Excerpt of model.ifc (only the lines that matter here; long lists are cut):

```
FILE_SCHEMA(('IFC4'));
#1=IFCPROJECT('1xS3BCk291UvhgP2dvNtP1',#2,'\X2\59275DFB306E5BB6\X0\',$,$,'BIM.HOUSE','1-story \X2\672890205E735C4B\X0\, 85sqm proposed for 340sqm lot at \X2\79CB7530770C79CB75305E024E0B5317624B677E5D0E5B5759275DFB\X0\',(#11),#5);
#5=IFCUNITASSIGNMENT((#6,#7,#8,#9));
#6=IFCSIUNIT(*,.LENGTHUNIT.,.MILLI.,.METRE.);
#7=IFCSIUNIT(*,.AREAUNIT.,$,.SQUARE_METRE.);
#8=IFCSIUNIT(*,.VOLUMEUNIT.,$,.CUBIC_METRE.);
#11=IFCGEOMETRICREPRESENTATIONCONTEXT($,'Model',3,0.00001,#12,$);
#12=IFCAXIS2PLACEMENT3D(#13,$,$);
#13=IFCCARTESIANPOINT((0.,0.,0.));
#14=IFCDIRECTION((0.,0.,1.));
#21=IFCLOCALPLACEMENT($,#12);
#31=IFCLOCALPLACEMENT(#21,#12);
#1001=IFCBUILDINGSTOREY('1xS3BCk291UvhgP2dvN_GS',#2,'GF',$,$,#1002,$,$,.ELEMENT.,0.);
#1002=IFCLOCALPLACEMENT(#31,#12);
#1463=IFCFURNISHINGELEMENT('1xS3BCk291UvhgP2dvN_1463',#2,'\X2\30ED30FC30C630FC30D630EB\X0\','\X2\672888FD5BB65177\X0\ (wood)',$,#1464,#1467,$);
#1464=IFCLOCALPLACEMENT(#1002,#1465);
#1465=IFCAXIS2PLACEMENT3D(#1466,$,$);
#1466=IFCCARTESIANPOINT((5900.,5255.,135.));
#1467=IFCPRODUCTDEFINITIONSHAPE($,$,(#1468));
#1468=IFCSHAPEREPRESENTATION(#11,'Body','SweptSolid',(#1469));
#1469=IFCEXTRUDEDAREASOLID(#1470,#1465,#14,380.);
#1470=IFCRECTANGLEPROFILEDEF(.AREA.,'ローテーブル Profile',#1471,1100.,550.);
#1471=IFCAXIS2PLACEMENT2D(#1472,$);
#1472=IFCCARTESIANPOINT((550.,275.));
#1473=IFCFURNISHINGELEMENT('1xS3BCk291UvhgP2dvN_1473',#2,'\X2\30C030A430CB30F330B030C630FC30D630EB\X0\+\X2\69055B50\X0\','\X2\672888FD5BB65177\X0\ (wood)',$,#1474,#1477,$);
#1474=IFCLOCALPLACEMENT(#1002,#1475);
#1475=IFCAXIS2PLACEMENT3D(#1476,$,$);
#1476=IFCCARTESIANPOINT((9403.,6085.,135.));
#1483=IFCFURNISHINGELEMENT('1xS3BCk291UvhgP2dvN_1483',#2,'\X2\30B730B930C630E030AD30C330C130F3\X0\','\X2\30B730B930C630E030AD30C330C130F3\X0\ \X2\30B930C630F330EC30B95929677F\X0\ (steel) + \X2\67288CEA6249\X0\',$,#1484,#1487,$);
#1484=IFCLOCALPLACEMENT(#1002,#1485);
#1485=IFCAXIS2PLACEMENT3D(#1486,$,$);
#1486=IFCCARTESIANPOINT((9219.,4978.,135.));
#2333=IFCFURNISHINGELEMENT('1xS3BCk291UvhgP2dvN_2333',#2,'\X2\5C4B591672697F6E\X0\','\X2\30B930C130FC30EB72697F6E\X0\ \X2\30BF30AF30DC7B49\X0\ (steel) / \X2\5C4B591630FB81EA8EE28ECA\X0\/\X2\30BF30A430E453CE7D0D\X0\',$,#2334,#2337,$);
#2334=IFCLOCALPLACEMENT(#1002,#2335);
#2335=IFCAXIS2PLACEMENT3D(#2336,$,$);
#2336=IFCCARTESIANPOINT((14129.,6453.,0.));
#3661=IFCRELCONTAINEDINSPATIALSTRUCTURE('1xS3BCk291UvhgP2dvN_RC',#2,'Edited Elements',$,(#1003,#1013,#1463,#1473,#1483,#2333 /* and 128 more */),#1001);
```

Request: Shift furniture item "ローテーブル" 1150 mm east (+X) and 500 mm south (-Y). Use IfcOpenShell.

```python
import ifcopenshell
import ifcopenshell.api.geometry
import ifcopenshell.util.placement
import ifcopenshell.util.unit

model = ifcopenshell.open("model.ifc")
unit_scale = ifcopenshell.util.unit.calculate_unit_scale(model)

item = model.by_id(1463)
matrix = ifcopenshell.util.placement.get_local_placement(item.ObjectPlacement)
matrix[0, 3] += 1.15 / unit_scale
matrix[1, 3] -= 0.5 / unit_scale
ifcopenshell.api.geometry.edit_object_placement(model, product=item, matrix=matrix, is_si=False)

print(ifcopenshell.util.placement.get_local_placement(item.ObjectPlacement).round(3) + 0.0)

model.write("model_updated.ifc")
```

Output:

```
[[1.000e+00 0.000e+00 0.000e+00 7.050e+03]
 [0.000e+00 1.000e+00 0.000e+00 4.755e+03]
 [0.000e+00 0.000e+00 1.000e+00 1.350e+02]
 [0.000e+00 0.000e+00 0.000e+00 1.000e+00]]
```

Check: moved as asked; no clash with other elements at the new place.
